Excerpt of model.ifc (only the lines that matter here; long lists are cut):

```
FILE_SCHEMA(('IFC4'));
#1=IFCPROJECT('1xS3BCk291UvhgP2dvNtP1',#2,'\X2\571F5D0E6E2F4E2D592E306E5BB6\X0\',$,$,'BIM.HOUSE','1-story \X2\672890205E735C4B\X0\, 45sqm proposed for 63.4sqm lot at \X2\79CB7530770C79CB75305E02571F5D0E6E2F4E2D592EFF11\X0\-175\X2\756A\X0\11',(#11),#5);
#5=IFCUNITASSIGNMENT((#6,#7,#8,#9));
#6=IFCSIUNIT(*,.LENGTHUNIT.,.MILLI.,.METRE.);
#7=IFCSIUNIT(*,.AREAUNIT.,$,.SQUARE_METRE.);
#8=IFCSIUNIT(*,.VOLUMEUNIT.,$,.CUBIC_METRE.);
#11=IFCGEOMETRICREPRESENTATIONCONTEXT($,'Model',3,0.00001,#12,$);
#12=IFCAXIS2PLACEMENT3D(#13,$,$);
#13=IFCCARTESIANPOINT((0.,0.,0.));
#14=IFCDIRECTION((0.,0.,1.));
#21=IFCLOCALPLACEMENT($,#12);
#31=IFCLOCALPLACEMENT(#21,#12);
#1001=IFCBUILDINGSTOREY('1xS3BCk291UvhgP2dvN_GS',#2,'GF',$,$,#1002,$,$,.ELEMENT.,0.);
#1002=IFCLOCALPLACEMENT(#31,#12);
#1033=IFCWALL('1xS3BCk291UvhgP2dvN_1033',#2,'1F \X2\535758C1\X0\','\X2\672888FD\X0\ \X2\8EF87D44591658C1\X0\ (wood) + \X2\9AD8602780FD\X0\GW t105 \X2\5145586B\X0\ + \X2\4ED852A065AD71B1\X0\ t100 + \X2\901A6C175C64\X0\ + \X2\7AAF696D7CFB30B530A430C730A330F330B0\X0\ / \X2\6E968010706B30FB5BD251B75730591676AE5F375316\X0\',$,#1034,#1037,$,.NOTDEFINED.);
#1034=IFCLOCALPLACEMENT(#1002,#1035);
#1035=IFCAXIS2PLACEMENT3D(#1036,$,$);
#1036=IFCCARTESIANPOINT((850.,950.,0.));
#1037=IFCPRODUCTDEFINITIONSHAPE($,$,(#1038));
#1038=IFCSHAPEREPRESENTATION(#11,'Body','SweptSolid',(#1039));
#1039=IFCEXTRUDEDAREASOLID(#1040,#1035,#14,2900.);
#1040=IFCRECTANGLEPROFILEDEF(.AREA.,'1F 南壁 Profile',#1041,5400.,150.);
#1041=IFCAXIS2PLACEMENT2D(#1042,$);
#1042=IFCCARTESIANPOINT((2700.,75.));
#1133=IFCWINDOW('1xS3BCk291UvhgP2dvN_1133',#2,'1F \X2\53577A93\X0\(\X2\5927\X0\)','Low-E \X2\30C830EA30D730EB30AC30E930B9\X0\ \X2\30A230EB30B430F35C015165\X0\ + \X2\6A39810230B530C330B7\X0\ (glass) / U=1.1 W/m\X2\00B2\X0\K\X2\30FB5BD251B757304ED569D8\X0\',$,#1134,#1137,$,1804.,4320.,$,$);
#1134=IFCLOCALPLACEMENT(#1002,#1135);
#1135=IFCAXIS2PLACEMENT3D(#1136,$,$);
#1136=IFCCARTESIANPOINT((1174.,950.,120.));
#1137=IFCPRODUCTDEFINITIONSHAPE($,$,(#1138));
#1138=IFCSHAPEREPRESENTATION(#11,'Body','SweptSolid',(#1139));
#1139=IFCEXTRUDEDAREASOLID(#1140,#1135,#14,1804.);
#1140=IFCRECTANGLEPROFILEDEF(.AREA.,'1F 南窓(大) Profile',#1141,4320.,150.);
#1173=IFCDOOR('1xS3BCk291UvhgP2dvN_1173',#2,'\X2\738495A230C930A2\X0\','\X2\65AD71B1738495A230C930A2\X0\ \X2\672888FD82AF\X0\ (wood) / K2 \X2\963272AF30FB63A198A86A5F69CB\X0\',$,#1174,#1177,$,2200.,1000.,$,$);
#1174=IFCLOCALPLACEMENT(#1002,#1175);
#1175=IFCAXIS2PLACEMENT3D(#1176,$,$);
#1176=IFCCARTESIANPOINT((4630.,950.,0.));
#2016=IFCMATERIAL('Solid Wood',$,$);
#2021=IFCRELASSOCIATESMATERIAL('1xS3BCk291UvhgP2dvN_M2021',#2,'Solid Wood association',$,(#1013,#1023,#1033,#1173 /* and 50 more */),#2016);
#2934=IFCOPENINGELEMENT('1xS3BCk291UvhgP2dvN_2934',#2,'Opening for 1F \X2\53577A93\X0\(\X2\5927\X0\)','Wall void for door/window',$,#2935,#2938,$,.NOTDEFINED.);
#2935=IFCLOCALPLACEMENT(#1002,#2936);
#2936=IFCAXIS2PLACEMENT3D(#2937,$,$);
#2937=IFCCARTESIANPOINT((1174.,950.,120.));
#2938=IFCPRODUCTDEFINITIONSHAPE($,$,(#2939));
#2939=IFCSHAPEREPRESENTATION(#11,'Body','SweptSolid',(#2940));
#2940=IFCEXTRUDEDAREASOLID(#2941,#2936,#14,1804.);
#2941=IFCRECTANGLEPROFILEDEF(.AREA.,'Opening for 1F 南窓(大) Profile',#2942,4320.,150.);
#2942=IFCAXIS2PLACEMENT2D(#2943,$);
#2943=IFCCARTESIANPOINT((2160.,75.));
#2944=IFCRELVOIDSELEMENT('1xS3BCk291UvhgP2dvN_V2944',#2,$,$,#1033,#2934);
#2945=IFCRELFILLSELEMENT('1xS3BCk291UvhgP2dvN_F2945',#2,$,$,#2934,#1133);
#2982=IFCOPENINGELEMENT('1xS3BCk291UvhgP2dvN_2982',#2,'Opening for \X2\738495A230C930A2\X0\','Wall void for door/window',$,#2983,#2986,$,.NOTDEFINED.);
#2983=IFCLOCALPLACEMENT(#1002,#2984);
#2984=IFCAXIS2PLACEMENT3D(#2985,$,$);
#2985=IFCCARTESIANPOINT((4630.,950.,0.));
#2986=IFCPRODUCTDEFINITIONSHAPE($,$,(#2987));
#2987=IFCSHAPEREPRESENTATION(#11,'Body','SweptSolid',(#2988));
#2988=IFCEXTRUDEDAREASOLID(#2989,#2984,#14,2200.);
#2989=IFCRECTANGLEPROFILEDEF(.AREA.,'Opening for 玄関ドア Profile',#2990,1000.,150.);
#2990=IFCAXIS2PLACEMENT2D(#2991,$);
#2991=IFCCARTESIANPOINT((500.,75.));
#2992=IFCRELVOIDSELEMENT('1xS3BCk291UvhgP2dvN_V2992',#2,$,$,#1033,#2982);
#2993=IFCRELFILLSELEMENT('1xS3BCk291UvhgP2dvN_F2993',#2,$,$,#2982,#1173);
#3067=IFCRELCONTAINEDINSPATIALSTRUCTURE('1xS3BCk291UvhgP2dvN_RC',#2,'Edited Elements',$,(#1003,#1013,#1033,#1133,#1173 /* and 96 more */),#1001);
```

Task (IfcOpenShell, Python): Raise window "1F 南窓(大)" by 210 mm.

```python
import numpy as np
import ifcopenshell
import ifcopenshell.api.geometry
import ifcopenshell.util.placement
import ifcopenshell.util.unit

model = ifcopenshell.open("model.ifc")
unit_scale = ifcopenshell.util.unit.calculate_unit_scale(model)

window = model.by_guid("1xS3BCk291UvhgP2dvN_1133")
opening = window.FillsVoids[0].RelatingOpeningElement
dz = 210.0

shift = np.array([0.0, 0.0, dz])
# The window is not placed relative to its opening, so move both.
for product in (opening, window):
    matrix = ifcopenshell.util.placement.get_local_placement(product.ObjectPlacement)
    matrix[:3, 3] += shift
    ifcopenshell.api.geometry.edit_object_placement(model, product=product, matrix=matrix, is_si=False)

print(f"moved by {dz * unit_scale:+.3f} m")

model.write("model-out.ifc")
```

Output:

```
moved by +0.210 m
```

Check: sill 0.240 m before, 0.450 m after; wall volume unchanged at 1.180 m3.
